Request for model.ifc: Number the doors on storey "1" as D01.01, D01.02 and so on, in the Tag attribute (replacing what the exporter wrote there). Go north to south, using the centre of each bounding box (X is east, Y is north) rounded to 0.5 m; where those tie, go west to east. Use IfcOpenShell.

First a look at what the model holds.

```python
import ifcopenshell
import ifcopenshell.util.element
import ifcopenshell.util.placement

model = ifcopenshell.open("model.ifc")
print(model.schema)
storey = next(s for s in model.by_type("IfcBuildingStorey") if s.Name == "1")
doors = [e for e in ifcopenshell.util.element.get_decomposition(storey) if e.is_a("IfcDoor")]
for e in sorted(doors, key=lambda e: e.id()):
    origin = ifcopenshell.util.placement.get_local_placement(e.ObjectPlacement)[:3, 3]
    print(e.id(), e.Tag, e.Name, origin.round(2) + 0.0, sep=" | ")
```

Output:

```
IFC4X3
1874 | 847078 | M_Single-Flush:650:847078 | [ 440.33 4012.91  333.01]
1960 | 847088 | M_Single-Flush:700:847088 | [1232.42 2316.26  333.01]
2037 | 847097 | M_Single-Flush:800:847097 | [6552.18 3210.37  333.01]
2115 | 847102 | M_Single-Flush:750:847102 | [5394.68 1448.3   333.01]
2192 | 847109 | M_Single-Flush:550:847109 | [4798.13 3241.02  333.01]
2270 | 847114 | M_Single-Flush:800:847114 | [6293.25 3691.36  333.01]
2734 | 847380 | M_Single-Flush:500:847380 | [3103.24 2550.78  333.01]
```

```python
import ifcopenshell
import ifcopenshell.geom
import ifcopenshell.util.element
import ifcopenshell.util.shape

model = ifcopenshell.open("model.ifc")
settings = ifcopenshell.geom.settings()
settings.set("use-world-coords", True)


def centre(element):
    shape = ifcopenshell.geom.create_shape(settings, element)
    return ifcopenshell.util.shape.get_bbox_centroid(shape.geometry)


storey = next(s for s in model.by_type("IfcBuildingStorey") if s.Name == "1")
doors = [e for e in ifcopenshell.util.element.get_decomposition(storey) if e.is_a("IfcDoor")]

# Insertion points can sit at a corner or the storey origin, so sort by the geometry (in metres).
centres = {e: centre(e) for e in doors}
doors.sort(key=lambda e: (-round(centres[e][1] / 0.5), centres[e][0]))

for i, e in enumerate(doors, start=1):
    number = f"D01.{i:02d}"
    e.Tag = number
    print(e.id(), number)

model.write("model_rev.ifc")
```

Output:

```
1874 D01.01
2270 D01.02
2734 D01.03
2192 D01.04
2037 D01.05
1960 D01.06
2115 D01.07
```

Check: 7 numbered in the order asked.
